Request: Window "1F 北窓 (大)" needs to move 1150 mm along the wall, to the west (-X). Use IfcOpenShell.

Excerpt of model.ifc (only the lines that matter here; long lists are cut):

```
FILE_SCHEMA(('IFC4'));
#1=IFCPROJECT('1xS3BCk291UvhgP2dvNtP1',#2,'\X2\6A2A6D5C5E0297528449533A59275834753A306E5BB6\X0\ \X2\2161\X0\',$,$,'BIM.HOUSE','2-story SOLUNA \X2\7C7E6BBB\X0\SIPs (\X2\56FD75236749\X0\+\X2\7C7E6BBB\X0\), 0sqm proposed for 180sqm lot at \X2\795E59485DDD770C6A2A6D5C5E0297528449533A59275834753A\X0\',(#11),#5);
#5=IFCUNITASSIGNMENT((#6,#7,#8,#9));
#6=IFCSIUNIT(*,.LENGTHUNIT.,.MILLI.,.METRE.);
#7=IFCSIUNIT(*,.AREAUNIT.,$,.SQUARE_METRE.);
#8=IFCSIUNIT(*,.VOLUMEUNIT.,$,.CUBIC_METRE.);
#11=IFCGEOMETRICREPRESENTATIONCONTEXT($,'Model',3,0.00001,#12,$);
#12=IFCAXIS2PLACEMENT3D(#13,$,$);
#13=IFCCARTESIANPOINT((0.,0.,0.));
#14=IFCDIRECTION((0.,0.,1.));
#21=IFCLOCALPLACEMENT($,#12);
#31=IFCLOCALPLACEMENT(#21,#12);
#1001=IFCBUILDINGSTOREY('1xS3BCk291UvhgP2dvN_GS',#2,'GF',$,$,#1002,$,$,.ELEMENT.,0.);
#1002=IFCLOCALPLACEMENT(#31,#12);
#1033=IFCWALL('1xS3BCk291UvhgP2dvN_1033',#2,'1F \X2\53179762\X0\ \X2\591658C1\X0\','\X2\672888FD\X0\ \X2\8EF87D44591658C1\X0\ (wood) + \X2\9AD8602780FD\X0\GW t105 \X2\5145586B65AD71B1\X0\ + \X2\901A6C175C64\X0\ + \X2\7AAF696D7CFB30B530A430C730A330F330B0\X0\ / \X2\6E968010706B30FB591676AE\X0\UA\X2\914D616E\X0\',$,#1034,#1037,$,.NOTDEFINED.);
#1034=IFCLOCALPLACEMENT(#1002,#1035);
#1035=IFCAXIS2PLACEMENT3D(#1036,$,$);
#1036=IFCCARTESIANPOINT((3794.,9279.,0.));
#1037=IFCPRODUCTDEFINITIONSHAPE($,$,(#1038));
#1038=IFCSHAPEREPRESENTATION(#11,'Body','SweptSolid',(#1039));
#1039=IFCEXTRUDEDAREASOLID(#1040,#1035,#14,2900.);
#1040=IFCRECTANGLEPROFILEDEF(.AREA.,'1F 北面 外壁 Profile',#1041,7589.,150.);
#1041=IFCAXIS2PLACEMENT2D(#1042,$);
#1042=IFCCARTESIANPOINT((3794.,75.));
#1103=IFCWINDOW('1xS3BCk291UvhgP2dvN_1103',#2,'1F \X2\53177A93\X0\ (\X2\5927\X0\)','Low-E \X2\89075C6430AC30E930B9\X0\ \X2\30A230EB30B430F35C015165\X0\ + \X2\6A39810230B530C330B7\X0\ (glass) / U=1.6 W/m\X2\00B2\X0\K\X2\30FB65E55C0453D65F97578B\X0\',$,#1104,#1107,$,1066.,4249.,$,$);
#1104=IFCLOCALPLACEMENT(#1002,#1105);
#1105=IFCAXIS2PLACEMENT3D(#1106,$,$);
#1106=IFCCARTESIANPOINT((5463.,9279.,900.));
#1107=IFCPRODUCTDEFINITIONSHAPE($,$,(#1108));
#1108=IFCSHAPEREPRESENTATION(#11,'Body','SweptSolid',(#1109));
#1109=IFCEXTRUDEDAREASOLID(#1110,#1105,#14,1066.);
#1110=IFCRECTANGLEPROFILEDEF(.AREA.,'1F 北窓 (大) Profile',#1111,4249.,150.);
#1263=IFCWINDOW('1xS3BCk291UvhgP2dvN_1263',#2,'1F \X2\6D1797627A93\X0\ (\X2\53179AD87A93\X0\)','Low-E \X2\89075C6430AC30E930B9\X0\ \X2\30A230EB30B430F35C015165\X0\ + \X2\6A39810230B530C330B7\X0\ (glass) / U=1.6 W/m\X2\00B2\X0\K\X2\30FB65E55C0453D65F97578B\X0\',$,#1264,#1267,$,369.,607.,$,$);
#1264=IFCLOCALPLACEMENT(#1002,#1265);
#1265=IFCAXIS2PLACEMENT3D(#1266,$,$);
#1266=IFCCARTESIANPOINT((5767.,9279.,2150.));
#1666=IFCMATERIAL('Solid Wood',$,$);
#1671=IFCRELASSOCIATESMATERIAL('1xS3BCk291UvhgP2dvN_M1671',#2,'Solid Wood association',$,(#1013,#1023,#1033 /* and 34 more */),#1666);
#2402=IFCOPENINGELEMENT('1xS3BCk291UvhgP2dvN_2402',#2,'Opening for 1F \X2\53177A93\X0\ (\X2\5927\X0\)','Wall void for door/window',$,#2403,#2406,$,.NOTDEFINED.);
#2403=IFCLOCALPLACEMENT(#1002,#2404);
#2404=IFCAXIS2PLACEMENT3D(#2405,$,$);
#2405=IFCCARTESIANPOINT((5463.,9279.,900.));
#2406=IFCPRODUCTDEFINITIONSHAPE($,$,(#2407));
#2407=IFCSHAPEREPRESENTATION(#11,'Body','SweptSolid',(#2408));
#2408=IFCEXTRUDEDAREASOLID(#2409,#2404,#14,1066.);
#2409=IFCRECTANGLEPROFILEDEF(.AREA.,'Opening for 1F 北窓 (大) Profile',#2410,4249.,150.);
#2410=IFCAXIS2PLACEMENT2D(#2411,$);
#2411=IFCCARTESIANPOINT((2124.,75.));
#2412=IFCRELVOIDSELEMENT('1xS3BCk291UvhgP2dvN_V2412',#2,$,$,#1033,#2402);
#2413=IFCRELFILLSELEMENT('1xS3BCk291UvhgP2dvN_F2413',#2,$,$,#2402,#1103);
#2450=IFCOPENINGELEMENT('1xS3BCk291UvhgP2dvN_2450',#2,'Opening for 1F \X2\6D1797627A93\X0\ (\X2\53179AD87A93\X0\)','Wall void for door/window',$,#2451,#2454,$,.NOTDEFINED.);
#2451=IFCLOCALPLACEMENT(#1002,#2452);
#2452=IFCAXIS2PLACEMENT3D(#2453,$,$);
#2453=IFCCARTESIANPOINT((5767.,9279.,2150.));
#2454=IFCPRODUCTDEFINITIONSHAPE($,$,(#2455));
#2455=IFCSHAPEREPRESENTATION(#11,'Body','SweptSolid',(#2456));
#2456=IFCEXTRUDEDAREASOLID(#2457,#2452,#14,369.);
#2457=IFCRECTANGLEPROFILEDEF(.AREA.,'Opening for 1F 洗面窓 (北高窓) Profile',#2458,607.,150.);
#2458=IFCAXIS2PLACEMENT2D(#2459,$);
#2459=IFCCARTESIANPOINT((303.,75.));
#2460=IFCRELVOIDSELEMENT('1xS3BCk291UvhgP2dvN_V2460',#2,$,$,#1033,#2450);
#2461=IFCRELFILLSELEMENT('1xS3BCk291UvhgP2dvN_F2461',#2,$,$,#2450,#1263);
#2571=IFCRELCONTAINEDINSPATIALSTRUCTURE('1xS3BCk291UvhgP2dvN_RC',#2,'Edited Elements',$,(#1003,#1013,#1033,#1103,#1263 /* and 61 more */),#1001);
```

```python
import ifcopenshell
import ifcopenshell.api.geometry
import ifcopenshell.util.placement
import ifcopenshell.util.unit

model = ifcopenshell.open("model.ifc")
unit_scale = ifcopenshell.util.unit.calculate_unit_scale(model)

window = model.by_guid("1xS3BCk291UvhgP2dvN_1103")
opening = window.FillsVoids[0].RelatingOpeningElement
wall = opening.VoidsElements[0].RelatingBuildingElement

wall_matrix = ifcopenshell.util.placement.get_local_placement(wall.ObjectPlacement)
shift = wall_matrix[:3, 0] * -1.15 / unit_scale
before = ifcopenshell.util.placement.get_local_placement(window.ObjectPlacement)[:3, 3].copy()

# The window is not placed relative to its opening, so move both.
for product in (opening, window):
    matrix = ifcopenshell.util.placement.get_local_placement(product.ObjectPlacement)
    matrix[:3, 3] += shift
    ifcopenshell.api.geometry.edit_object_placement(model, product=product, matrix=matrix, is_si=False)

after = ifcopenshell.util.placement.get_local_placement(window.ObjectPlacement)[:3, 3]
print("window moved by", (after - before).round(3) + 0.0)

model.write("model_rev.ifc")
```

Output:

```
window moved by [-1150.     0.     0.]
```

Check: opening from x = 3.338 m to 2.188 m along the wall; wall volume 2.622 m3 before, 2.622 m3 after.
